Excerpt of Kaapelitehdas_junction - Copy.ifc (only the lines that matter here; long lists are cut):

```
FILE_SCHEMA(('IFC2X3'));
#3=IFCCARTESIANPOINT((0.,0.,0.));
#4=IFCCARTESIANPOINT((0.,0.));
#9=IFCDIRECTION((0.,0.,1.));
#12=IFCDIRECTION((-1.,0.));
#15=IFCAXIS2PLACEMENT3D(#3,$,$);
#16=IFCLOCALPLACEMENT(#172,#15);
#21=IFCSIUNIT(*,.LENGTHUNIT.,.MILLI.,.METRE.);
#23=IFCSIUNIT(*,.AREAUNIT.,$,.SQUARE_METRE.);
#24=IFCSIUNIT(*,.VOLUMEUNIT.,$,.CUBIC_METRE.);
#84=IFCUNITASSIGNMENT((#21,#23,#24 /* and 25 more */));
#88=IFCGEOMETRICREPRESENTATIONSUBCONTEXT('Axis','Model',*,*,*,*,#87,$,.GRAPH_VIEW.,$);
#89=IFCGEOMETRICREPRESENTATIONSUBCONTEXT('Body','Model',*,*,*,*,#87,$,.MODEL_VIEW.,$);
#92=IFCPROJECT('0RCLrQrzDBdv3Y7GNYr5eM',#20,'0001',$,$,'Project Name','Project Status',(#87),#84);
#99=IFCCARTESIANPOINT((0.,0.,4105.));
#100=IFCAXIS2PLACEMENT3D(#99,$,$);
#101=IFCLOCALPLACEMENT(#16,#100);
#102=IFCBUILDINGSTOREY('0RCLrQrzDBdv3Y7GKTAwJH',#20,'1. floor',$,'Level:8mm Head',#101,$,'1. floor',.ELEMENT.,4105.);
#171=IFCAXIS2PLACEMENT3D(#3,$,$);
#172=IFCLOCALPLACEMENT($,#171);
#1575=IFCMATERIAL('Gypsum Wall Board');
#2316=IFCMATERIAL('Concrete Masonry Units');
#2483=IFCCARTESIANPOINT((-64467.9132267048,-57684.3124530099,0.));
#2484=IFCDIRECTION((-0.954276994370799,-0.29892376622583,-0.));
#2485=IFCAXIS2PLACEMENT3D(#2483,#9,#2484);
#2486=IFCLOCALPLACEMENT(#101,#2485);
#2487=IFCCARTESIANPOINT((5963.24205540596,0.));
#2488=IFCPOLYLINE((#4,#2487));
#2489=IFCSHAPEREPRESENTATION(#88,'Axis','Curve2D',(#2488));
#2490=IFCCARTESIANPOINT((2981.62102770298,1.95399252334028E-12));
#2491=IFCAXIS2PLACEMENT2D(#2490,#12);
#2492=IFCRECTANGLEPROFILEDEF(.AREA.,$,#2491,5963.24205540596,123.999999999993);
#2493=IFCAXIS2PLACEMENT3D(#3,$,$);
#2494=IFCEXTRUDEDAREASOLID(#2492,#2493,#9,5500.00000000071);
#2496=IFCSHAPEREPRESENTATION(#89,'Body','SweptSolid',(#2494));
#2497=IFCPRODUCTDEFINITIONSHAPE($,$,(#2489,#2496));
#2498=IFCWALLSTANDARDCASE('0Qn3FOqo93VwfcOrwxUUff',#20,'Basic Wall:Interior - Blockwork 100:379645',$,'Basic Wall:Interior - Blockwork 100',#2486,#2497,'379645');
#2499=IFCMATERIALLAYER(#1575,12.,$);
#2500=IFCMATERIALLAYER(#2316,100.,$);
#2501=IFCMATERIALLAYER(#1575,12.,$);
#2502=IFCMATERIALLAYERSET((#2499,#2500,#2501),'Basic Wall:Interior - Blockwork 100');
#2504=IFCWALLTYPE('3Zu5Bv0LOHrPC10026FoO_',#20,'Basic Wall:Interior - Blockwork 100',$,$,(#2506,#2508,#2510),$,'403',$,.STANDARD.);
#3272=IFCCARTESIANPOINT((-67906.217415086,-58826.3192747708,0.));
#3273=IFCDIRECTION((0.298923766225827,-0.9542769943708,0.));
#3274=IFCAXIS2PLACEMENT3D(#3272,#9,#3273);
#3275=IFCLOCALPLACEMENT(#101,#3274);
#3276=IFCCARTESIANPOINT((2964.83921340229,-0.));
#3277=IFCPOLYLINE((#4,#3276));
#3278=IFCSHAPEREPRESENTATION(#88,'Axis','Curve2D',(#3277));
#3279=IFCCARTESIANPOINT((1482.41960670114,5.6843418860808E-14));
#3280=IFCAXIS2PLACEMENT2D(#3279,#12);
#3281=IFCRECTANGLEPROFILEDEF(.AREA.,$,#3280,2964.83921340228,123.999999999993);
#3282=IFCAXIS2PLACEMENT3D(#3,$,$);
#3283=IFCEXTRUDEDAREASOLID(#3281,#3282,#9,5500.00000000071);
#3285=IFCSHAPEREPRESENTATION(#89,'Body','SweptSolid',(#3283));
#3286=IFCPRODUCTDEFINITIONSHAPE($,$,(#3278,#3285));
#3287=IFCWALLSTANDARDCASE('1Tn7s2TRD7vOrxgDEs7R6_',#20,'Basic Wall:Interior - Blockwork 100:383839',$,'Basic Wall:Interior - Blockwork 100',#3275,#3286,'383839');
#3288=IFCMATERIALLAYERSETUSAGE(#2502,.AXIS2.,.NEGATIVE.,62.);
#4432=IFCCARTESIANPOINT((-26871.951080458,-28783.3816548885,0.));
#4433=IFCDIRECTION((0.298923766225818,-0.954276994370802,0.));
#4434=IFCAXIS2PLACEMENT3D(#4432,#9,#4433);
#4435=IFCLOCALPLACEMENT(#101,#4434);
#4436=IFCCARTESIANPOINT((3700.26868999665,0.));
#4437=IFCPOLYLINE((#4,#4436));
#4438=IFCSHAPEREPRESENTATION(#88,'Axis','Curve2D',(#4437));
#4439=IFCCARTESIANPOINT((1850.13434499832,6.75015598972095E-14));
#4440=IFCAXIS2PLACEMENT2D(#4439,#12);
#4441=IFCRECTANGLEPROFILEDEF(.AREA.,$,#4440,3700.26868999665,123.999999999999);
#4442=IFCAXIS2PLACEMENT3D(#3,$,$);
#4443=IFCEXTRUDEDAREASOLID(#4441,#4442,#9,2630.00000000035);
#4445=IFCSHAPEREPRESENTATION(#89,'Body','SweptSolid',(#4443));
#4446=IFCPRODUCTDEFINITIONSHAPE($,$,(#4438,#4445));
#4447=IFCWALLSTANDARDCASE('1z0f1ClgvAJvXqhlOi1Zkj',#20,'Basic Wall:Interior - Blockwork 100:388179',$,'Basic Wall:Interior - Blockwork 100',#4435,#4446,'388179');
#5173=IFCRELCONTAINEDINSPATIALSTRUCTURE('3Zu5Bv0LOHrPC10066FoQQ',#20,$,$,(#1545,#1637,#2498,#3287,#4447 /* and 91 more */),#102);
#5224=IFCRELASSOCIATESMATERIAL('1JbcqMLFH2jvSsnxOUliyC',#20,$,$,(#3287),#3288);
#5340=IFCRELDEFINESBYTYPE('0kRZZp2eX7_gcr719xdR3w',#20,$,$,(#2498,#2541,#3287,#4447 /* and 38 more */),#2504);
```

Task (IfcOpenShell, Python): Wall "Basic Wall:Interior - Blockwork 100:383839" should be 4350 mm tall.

```python
import ifcopenshell
import ifcopenshell.geom
import ifcopenshell.util.representation
import ifcopenshell.util.shape
import ifcopenshell.util.unit

model = ifcopenshell.open("Kaapelitehdas_junction - Copy.ifc")
unit_scale = ifcopenshell.util.unit.calculate_unit_scale(model)
settings = ifcopenshell.geom.settings()


def volume(element):
    """Net volume in cubic metres, openings subtracted."""
    shape = ifcopenshell.geom.create_shape(settings, element)
    return ifcopenshell.util.shape.get_volume(shape.geometry)


wall = model.by_guid("1Tn7s2TRD7vOrxgDEs7R6_")
before = volume(wall)

body = ifcopenshell.util.representation.get_representation(wall, "Model", "Body")
solid = body.Items[0]
old_height = solid.Depth
solid.Depth = 4.35 / unit_scale
after = volume(wall)

print(f"height {old_height:g} -> {solid.Depth:g}, volume {before:.3f} -> {after:.3f} m3")

model.write("Kaapelitehdas_junction - Copy_edited.ifc")
```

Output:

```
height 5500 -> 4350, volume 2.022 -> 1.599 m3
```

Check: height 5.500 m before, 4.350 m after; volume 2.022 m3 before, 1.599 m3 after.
